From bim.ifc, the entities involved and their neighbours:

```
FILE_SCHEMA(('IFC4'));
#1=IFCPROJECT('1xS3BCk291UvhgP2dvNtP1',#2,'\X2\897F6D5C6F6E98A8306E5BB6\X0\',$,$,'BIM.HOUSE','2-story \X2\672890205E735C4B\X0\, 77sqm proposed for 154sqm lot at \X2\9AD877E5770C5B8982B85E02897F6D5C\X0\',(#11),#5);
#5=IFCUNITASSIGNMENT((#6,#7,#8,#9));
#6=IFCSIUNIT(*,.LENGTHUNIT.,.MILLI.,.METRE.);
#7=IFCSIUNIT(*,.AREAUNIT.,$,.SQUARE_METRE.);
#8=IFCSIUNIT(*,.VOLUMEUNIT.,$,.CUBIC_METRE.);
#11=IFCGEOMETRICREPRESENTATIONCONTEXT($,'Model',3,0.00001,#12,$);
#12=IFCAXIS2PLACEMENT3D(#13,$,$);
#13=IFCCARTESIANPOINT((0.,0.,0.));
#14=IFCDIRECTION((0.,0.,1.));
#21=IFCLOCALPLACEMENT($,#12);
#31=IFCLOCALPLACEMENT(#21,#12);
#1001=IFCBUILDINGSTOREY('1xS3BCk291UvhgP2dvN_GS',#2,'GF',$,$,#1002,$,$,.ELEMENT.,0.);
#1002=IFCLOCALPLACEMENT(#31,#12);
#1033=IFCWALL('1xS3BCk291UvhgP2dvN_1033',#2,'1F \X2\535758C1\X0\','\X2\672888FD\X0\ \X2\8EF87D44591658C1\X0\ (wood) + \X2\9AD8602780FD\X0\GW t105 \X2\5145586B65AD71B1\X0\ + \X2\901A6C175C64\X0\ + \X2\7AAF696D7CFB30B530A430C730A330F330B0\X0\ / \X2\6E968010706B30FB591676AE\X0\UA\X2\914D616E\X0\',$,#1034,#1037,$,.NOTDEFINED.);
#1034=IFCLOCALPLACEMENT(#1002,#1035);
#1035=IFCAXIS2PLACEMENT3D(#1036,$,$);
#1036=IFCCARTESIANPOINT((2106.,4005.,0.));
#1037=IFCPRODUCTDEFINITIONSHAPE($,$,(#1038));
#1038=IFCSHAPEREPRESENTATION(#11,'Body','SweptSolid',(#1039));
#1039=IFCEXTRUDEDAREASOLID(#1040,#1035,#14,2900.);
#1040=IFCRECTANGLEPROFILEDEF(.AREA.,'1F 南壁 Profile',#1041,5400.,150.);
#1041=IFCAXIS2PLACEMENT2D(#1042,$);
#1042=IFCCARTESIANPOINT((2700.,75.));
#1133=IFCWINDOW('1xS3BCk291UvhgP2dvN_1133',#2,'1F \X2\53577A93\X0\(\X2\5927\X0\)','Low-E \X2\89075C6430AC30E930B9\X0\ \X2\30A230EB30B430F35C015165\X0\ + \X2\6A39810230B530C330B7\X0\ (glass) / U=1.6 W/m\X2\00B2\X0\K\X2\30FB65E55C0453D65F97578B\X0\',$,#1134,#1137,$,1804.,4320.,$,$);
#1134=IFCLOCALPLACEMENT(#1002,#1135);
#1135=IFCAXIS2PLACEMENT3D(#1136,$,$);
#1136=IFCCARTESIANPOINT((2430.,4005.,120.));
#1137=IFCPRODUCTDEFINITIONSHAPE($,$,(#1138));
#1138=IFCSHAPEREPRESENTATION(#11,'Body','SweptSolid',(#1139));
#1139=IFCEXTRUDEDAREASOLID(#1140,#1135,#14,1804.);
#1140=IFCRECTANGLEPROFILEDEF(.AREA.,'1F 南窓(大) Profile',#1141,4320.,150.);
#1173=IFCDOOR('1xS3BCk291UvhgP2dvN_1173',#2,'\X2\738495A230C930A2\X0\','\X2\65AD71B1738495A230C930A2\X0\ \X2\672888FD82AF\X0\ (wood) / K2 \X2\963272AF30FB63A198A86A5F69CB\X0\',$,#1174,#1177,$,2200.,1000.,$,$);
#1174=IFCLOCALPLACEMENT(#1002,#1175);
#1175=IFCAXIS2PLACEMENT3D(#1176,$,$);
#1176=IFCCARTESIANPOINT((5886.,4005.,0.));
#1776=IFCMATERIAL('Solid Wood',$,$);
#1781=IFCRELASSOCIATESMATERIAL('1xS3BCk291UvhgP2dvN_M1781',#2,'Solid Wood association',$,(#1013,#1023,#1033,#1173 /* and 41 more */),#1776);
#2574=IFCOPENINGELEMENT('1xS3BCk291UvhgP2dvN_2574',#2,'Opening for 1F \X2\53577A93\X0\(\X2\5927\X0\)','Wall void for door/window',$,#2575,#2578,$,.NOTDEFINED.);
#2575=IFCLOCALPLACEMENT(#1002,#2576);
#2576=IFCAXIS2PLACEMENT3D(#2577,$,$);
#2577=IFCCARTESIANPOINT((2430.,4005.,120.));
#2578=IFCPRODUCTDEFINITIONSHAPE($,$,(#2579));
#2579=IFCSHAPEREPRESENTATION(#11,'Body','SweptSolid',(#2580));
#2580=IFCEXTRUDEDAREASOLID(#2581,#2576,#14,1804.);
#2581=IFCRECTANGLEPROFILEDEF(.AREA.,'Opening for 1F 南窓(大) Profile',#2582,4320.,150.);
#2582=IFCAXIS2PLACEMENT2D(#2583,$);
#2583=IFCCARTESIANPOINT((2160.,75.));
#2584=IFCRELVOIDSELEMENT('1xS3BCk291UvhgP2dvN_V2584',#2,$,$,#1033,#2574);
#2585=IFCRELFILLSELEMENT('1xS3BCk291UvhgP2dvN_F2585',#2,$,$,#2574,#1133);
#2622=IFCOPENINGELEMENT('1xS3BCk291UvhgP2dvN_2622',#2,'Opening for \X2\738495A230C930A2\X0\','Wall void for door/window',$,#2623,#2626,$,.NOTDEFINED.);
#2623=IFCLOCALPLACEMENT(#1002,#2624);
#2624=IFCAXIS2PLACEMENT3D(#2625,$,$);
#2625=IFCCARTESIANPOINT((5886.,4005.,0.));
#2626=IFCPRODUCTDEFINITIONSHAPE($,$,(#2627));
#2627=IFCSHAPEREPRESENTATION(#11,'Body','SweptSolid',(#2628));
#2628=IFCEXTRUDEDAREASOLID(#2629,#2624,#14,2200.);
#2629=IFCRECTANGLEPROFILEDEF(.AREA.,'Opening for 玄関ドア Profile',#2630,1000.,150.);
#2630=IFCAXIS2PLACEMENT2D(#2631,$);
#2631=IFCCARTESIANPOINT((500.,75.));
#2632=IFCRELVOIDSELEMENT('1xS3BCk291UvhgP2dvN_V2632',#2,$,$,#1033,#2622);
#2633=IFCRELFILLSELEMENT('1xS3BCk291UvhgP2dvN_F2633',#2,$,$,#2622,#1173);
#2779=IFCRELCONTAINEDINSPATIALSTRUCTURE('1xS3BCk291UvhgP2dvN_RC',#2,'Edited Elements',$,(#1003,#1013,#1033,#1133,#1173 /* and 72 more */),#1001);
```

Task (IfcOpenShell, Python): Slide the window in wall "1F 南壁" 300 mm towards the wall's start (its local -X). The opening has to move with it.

```python
import ifcopenshell
import ifcopenshell.api.geometry
import ifcopenshell.util.placement
import ifcopenshell.util.unit

model = ifcopenshell.open("bim.ifc")
unit_scale = ifcopenshell.util.unit.calculate_unit_scale(model)

window = model.by_guid("1xS3BCk291UvhgP2dvN_1133")
opening = window.FillsVoids[0].RelatingOpeningElement
wall = opening.VoidsElements[0].RelatingBuildingElement

wall_matrix = ifcopenshell.util.placement.get_local_placement(wall.ObjectPlacement)
shift = wall_matrix[:3, 0] * -0.3 / unit_scale
before = ifcopenshell.util.placement.get_local_placement(window.ObjectPlacement)[:3, 3].copy()

# The window is not placed relative to its opening, so move both.
for product in (opening, window):
    matrix = ifcopenshell.util.placement.get_local_placement(product.ObjectPlacement)
    matrix[:3, 3] += shift
    ifcopenshell.api.geometry.edit_object_placement(model, product=product, matrix=matrix, is_si=False)

after = ifcopenshell.util.placement.get_local_placement(window.ObjectPlacement)[:3, 3]
print("window moved by", (after - before).round(3) + 0.0)

model.write("bim-out.ifc")
```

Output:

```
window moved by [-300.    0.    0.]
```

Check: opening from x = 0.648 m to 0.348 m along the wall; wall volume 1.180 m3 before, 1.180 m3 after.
